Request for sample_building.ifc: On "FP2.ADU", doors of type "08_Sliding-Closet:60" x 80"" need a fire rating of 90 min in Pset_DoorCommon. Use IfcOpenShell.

First a look at what the model holds.

```python
import ifcopenshell
import ifcopenshell.util.element

model = ifcopenshell.open("sample_building.ifc")
print(model.schema)
storey = next(s for s in model.by_type("IfcBuildingStorey") if s.Name == "FP2.ADU")
doors = [e for e in ifcopenshell.util.element.get_decomposition(storey) if e.is_a("IfcDoor")]
seen = {}
for e in doors:
    element_type = ifcopenshell.util.element.get_type(e)
    key = (element_type.Name if element_type != e and element_type else None, ifcopenshell.util.element.get_pset(e, "Pset_DoorCommon", "FireRating"))
    seen[key] = seen.get(key, 0) + 1
for (name, value), count in sorted(seen.items(), key=str):
    print(count, "x", name, "|", value)
```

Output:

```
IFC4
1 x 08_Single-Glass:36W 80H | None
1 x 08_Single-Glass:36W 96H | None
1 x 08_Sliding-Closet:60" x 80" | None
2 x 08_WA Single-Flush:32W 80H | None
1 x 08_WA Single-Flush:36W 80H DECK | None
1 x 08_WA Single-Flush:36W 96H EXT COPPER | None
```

```python
import ifcopenshell
import ifcopenshell.api.pset
import ifcopenshell.util.element

model = ifcopenshell.open("sample_building.ifc")

storey = next(s for s in model.by_type("IfcBuildingStorey") if s.Name == "FP2.ADU")
doors = [e for e in ifcopenshell.util.element.get_decomposition(storey) if e.is_a("IfcDoor")]

count = 0
for e in doors:
    element_type = ifcopenshell.util.element.get_type(e)
    if element_type in (None, e) or element_type.Name != '08_Sliding-Closet:60" x 80"':
        continue
    # add_pset returns the element's existing set when there is one.
    pset = ifcopenshell.api.pset.add_pset(model, product=e, name="Pset_DoorCommon")
    ifcopenshell.api.pset.edit_pset(model, pset=pset, properties={"FireRating": "90 min"})
    count += 1

print(count, "doors updated")

model.write("sample_building-out.ifc")
```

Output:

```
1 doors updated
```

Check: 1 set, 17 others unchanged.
